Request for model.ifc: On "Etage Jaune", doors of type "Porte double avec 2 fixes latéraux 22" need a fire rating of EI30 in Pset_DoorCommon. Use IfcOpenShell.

First a look at what the model holds.

```python
import ifcopenshell
import ifcopenshell.util.element

model = ifcopenshell.open("model.ifc")
print(model.schema)
storey = next(s for s in model.by_type("IfcBuildingStorey") if s.Name == "Etage Jaune")
doors = [e for e in ifcopenshell.util.element.get_decomposition(storey) if e.is_a("IfcDoor")]
seen = {}
for e in doors:
    element_type = ifcopenshell.util.element.get_type(e)
    key = (element_type.Name if element_type != e and element_type else None, ifcopenshell.util.element.get_pset(e, "Pset_DoorCommon", "FireRating"))
    seen[key] = seen.get(key, 0) + 1
for (name, value), count in sorted(seen.items(), key=str):
    print(count, "x", name, "|", value)
```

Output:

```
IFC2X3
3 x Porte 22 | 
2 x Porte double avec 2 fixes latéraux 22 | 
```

```python
import ifcopenshell
import ifcopenshell.api.pset
import ifcopenshell.util.element

model = ifcopenshell.open("model.ifc")

storey = next(s for s in model.by_type("IfcBuildingStorey") if s.Name == "Etage Jaune")
doors = [e for e in ifcopenshell.util.element.get_decomposition(storey) if e.is_a("IfcDoor")]

count = 0
for e in doors:
    element_type = ifcopenshell.util.element.get_type(e)
    if element_type in (None, e) or element_type.Name != "Porte double avec 2 fixes latéraux 22":
        continue
    # add_pset returns the element's existing set when there is one.
    pset = ifcopenshell.api.pset.add_pset(model, product=e, name="Pset_DoorCommon")
    ifcopenshell.api.pset.edit_pset(model, pset=pset, properties={"FireRating": "EI30"})
    count += 1

print(count, "doors updated")

model.write("model-out.ifc")
```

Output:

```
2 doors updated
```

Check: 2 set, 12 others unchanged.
